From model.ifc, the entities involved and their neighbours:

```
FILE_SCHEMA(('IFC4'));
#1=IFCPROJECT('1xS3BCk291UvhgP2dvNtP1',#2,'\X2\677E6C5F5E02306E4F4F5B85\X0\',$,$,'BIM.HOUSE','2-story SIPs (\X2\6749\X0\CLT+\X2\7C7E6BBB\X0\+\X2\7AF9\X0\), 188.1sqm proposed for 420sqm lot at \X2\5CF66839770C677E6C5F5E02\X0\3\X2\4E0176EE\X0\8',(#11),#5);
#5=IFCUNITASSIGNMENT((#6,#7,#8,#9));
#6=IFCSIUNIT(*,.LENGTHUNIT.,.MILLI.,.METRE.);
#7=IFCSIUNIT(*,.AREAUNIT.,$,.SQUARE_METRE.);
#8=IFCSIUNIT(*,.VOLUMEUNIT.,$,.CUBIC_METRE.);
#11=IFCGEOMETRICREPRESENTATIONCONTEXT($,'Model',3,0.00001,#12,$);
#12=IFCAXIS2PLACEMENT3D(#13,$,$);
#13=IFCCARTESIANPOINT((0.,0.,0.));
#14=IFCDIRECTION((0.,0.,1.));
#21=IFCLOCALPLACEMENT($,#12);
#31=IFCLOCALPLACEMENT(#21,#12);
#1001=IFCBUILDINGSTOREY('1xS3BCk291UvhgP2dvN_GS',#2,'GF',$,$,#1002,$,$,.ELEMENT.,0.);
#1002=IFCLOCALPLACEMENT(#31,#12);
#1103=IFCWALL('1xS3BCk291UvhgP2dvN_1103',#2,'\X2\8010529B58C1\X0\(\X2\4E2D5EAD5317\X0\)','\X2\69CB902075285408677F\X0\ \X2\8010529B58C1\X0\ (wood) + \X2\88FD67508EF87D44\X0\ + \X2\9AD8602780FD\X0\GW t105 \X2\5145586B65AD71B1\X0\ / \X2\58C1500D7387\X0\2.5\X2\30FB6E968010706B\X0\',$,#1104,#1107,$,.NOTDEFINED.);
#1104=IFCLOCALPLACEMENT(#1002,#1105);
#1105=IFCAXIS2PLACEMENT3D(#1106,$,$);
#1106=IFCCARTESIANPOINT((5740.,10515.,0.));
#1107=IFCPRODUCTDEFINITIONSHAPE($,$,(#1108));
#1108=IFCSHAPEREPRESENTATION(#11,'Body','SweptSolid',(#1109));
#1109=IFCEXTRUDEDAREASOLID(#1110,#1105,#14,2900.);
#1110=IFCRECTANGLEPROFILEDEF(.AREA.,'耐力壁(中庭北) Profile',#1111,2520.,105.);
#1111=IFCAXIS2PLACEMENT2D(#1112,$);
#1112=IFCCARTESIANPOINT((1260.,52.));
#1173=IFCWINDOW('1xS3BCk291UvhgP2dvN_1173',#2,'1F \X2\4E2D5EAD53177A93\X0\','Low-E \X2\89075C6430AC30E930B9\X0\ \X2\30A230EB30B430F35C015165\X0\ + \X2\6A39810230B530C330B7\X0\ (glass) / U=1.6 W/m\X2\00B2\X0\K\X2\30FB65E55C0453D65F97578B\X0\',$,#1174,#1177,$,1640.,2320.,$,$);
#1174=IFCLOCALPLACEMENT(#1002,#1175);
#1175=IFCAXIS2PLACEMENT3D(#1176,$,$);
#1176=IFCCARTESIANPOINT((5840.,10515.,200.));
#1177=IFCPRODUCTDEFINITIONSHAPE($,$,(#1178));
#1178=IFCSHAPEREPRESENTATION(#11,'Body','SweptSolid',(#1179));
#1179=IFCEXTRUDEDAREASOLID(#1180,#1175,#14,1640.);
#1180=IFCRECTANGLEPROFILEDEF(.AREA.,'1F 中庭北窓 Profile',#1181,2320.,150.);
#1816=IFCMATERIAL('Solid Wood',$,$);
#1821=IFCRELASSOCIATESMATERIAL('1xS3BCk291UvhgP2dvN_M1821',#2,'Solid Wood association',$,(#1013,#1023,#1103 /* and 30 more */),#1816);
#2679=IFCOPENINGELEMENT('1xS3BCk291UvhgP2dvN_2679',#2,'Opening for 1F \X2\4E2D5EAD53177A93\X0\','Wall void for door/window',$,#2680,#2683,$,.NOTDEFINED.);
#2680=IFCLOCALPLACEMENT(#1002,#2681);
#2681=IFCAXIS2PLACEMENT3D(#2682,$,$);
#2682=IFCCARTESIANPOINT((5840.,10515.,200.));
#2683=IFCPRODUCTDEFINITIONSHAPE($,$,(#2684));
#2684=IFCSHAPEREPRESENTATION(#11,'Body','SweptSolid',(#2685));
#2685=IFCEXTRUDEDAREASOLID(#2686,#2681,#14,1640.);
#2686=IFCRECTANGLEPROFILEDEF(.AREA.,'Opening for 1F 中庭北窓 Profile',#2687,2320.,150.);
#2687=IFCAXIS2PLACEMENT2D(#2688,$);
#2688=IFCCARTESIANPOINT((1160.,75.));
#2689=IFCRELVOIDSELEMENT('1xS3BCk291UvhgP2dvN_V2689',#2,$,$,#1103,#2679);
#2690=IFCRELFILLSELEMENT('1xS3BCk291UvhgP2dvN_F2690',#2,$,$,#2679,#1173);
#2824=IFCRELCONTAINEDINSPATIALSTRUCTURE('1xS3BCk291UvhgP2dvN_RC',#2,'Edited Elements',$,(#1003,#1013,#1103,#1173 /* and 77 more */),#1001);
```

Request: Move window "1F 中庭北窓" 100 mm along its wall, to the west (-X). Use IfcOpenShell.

```python
import ifcopenshell
import ifcopenshell.api.geometry
import ifcopenshell.util.placement
import ifcopenshell.util.unit

model = ifcopenshell.open("model.ifc")
unit_scale = ifcopenshell.util.unit.calculate_unit_scale(model)

window = model.by_guid("1xS3BCk291UvhgP2dvN_1173")
opening = window.FillsVoids[0].RelatingOpeningElement
wall = opening.VoidsElements[0].RelatingBuildingElement

wall_matrix = ifcopenshell.util.placement.get_local_placement(wall.ObjectPlacement)
shift = wall_matrix[:3, 0] * -0.1 / unit_scale
before = ifcopenshell.util.placement.get_local_placement(window.ObjectPlacement)[:3, 3].copy()

# The window is not placed relative to its opening, so move both.
for product in (opening, window):
    matrix = ifcopenshell.util.placement.get_local_placement(product.ObjectPlacement)
    matrix[:3, 3] += shift
    ifcopenshell.api.geometry.edit_object_placement(model, product=product, matrix=matrix, is_si=False)

after = ifcopenshell.util.placement.get_local_placement(window.ObjectPlacement)[:3, 3]
print("window moved by", (after - before).round(3) + 0.0)

model.write("model_updated.ifc")
```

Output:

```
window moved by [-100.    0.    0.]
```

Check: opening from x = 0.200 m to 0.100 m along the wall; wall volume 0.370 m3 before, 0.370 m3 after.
